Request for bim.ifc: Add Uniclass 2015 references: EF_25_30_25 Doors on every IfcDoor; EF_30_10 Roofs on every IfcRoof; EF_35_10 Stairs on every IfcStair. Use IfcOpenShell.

First a look at what the model holds.

```python
import ifcopenshell

model = ifcopenshell.open("bim.ifc")
print(model.schema)
print("classifications:", [c.Name for c in model.by_type("IfcClassification")])
for ifc_class in ("IfcDoor", "IfcRoof", "IfcStair", "IfcWall", "IfcWindow"):
    print(ifc_class, len(model.by_type(ifc_class)))
```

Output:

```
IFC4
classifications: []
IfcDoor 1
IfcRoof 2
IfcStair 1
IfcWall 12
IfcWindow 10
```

```python
import ifcopenshell
import ifcopenshell.api.classification

model = ifcopenshell.open("bim.ifc")

system = ifcopenshell.api.classification.add_classification(model, classification="Uniclass 2015")

codes = {
    "IfcDoor": ("EF_25_30_25", "Doors"),
    "IfcRoof": ("EF_30_10", "Roofs"),
    "IfcStair": ("EF_35_10", "Stairs"),
}
for ifc_class, (code, name) in codes.items():
    products = model.by_type(ifc_class)
    ifcopenshell.api.classification.add_reference(
        model, products=products, classification=system, identification=code, name=name
    )
    print(code, len(products))

model.write("bim-out.ifc")
```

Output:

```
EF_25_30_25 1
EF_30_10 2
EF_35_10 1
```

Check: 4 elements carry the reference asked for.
